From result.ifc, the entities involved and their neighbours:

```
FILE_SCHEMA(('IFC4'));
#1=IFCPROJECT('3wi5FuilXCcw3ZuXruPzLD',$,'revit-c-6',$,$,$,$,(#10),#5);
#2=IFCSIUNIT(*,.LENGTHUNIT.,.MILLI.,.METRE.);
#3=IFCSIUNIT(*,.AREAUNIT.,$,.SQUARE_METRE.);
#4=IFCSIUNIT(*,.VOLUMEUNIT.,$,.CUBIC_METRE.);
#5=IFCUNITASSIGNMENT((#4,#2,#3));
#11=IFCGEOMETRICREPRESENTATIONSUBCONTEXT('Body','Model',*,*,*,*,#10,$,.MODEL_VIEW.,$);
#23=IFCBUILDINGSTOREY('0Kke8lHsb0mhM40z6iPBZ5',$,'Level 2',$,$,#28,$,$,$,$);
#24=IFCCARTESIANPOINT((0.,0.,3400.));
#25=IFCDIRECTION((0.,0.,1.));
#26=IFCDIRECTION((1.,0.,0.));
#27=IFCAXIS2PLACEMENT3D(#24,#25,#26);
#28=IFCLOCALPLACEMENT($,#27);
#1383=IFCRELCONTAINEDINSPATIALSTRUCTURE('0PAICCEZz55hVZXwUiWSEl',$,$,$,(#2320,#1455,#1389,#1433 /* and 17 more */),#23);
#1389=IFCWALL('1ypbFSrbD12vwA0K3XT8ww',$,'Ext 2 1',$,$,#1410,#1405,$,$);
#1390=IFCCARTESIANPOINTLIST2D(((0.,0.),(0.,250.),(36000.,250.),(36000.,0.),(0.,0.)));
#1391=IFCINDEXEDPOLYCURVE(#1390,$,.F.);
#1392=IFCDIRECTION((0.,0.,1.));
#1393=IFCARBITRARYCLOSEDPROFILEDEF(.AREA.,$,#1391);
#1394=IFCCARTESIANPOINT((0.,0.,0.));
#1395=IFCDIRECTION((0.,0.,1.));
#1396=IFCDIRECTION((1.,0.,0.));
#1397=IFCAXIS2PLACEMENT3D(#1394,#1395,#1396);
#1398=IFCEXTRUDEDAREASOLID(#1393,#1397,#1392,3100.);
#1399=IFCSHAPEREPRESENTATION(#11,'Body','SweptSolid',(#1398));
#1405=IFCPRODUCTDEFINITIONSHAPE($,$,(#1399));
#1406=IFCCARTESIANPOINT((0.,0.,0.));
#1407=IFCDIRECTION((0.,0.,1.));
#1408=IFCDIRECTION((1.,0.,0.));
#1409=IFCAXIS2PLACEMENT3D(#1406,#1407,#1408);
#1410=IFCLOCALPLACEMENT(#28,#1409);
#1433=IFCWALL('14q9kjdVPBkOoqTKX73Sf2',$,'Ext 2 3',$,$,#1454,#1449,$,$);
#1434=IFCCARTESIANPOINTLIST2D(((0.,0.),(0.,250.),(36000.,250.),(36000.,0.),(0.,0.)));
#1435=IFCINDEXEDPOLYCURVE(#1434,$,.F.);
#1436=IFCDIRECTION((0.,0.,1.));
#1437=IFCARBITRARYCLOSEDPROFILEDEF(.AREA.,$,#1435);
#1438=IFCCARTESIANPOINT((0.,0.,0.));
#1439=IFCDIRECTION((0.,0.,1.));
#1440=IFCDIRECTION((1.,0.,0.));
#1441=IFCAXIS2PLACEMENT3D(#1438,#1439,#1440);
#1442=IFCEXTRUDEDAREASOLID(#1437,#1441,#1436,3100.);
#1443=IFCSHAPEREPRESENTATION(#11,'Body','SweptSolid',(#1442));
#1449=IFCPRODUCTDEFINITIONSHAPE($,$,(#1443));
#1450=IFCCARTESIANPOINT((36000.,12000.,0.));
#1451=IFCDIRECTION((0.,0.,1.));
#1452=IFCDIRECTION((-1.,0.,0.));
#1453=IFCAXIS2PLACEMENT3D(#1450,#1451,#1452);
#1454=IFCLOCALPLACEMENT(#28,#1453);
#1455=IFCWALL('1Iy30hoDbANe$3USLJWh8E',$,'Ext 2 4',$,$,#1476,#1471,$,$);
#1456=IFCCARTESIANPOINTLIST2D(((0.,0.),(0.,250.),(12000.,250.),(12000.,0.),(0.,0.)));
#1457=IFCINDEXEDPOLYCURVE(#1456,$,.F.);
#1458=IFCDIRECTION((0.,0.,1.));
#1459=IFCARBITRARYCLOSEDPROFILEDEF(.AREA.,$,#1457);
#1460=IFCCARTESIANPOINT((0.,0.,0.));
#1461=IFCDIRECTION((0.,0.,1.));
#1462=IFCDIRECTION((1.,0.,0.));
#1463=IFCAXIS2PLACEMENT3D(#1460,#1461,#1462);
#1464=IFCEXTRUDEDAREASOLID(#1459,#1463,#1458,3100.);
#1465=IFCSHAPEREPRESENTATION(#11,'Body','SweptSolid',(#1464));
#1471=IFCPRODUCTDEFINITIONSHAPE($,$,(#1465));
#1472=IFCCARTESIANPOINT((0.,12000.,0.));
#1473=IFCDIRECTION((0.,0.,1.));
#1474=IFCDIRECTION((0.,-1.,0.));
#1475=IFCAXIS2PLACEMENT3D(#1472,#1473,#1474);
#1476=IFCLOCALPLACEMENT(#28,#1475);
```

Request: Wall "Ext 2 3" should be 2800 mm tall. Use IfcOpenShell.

```python
import ifcopenshell
import ifcopenshell.geom
import ifcopenshell.util.representation
import ifcopenshell.util.shape

model = ifcopenshell.open("result.ifc")
settings = ifcopenshell.geom.settings()


def volume(element):
    """Net volume in cubic metres, openings subtracted."""
    shape = ifcopenshell.geom.create_shape(settings, element)
    return ifcopenshell.util.shape.get_volume(shape.geometry)


wall = model.by_guid("14q9kjdVPBkOoqTKX73Sf2")
before = volume(wall)

body = ifcopenshell.util.representation.get_representation(wall, "Model", "Body")
solid = body.Items[0]
old_height = solid.Depth
solid.Depth = 2800.0
after = volume(wall)

print(f"height {old_height:g} -> {solid.Depth:g}, volume {before:.3f} -> {after:.3f} m3")

model.write("result_v2.ifc")
```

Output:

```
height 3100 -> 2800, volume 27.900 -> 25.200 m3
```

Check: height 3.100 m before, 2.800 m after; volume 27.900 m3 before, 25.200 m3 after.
